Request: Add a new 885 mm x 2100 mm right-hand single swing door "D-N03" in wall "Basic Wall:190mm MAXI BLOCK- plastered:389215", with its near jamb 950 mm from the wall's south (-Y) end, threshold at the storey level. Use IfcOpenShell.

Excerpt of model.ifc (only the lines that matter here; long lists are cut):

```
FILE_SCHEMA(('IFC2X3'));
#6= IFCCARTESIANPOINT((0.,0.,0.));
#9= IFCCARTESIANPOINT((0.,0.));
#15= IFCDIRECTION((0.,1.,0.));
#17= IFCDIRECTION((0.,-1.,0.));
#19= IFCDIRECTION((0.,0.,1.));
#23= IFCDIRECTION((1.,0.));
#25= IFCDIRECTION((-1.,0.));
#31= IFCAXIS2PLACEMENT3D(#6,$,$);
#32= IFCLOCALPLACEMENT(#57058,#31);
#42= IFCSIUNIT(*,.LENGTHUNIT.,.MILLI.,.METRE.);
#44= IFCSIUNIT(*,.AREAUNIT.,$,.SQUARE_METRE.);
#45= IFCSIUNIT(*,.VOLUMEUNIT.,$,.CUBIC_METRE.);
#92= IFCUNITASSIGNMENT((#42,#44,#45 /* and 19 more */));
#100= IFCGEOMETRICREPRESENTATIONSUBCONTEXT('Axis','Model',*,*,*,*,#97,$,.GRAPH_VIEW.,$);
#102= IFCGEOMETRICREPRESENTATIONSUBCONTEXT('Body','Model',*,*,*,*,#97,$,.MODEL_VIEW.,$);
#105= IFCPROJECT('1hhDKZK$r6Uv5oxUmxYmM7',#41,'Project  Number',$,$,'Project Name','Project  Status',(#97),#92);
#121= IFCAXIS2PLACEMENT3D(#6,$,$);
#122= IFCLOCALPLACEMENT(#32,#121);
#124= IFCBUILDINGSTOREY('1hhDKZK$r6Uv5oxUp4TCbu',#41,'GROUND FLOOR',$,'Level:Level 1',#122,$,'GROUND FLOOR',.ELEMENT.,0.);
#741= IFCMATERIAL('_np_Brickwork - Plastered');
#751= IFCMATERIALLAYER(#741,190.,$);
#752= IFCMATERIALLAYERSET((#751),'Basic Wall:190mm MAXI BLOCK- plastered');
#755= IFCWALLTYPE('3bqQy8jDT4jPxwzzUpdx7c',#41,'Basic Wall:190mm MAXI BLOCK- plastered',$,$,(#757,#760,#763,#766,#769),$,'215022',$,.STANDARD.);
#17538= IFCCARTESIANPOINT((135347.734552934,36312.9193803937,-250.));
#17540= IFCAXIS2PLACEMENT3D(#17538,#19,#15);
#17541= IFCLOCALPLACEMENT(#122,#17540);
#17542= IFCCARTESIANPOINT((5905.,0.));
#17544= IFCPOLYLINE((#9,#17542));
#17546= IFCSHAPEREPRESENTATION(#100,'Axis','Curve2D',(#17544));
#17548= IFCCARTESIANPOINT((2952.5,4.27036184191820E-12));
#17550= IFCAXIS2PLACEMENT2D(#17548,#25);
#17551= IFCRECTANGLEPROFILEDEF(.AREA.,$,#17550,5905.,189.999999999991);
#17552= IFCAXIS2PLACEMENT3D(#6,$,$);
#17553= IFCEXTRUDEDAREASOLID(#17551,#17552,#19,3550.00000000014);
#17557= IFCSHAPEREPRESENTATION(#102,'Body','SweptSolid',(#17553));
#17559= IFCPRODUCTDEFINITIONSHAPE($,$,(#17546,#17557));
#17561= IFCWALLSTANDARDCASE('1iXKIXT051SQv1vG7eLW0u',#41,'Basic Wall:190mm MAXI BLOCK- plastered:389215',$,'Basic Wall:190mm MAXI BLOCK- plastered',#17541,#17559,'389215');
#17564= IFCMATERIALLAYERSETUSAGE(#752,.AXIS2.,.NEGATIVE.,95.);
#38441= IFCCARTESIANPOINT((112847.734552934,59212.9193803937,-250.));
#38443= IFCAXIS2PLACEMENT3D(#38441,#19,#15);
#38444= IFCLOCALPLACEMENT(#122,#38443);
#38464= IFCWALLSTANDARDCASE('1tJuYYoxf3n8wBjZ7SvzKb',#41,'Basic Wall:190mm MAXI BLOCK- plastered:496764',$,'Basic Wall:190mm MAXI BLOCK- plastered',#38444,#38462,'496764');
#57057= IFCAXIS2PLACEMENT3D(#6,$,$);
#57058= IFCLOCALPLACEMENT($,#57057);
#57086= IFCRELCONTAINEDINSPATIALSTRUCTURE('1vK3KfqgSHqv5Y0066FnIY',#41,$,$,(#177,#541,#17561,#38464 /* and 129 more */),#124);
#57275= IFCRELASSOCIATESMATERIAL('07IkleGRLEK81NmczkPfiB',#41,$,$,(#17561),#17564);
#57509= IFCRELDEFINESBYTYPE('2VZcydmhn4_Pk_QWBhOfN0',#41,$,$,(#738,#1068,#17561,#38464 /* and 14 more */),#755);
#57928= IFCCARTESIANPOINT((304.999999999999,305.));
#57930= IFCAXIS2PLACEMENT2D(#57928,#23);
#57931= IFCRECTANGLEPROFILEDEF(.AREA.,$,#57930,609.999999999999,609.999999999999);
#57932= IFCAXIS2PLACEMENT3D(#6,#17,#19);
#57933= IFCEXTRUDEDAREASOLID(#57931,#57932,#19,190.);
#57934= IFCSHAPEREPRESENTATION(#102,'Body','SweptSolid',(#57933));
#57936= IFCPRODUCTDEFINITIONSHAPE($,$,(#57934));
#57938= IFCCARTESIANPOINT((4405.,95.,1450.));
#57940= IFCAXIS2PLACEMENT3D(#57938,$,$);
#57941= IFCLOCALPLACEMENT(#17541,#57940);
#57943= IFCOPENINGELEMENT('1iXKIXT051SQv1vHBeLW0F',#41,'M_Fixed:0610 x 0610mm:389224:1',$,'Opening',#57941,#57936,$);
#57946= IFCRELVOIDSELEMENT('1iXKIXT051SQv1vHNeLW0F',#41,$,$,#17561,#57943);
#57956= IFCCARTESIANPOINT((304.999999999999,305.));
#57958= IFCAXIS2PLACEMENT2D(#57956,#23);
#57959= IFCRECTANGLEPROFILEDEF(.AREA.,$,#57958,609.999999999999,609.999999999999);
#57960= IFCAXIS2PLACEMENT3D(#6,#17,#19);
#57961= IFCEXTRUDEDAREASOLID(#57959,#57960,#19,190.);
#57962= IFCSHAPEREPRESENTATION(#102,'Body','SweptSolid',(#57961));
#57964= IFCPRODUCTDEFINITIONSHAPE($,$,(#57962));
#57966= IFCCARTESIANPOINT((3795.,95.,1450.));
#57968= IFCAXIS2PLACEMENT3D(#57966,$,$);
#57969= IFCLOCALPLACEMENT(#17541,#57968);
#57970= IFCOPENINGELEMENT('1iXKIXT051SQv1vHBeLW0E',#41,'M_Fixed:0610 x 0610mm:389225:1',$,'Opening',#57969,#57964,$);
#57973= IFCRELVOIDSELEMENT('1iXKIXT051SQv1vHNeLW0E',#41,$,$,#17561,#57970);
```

```python
import numpy as np
import ifcopenshell
import ifcopenshell.api.feature
import ifcopenshell.api.geometry
import ifcopenshell.api.root
import ifcopenshell.api.spatial
import ifcopenshell.api.type
import ifcopenshell.geom
import ifcopenshell.util.element
import ifcopenshell.util.placement
import ifcopenshell.util.representation
import ifcopenshell.util.shape
import ifcopenshell.util.unit

model = ifcopenshell.open("model.ifc")
unit_scale = ifcopenshell.util.unit.calculate_unit_scale(model)
settings = ifcopenshell.geom.settings()


def volume(element):
    """Net volume in cubic metres, openings subtracted."""
    shape = ifcopenshell.geom.create_shape(settings, element)
    return ifcopenshell.util.shape.get_volume(shape.geometry)


wall = model.by_id(17561)
storey = ifcopenshell.util.element.get_container(wall, ifc_class="IfcBuildingStorey")
context = ifcopenshell.util.representation.get_context(model, "Model", "Body", "MODEL_VIEW")
before = volume(wall)

width, height, from_end, sill = 0.885, 2.1, 0.95, 0.0  # metres

# The wall runs along its own X axis, and the end named is its -X end.
wall_shape = ifcopenshell.geom.create_shape(settings, wall)
x, y, z = ifcopenshell.util.shape.get_vertices(wall_shape.geometry).T
start = x.min() + from_end
face, thickness = float(y.min()), float(y.max() - y.min())
wall_matrix = ifcopenshell.util.placement.get_local_placement(wall.ObjectPlacement)
level = ifcopenshell.util.placement.get_local_placement(storey.ObjectPlacement)[2, 3]


def in_wall(x, y):
    """Placement at x, y metres in the wall's axes, at sill height."""
    matrix = wall_matrix.copy()
    matrix[:, 3] = wall_matrix @ np.array([x / unit_scale, y / unit_scale, 0.0, 1.0])
    matrix[2, 3] = level + sill / unit_scale
    return matrix


# Opening: a box that overshoots both wall faces by 50 mm.
opening = ifcopenshell.api.root.create_entity(model, ifc_class="IfcOpeningElement")
box = ifcopenshell.api.geometry.add_wall_representation(
    model, context=context, length=width, height=height, thickness=thickness + 0.1
)
ifcopenshell.api.geometry.assign_representation(model, product=opening, representation=box)
ifcopenshell.api.geometry.edit_object_placement(model, product=opening, matrix=in_wall(start, face - 0.05), is_si=False)
ifcopenshell.api.feature.add_feature(model, feature=opening, element=wall)

door = ifcopenshell.api.root.create_entity(model, ifc_class="IfcDoor", name="D-N03")
door.OverallWidth, door.OverallHeight = width / unit_scale, height / unit_scale
body = ifcopenshell.api.geometry.add_door_representation(
    model,
    context=context,
    overall_width=door.OverallWidth,
    overall_height=door.OverallHeight,
    operation_type="SINGLE_SWING_RIGHT",
    lining_properties={"LiningDepth": thickness / unit_scale, "ThresholdDepth": thickness / unit_scale},
)
ifcopenshell.api.geometry.assign_representation(model, product=door, representation=body)
ifcopenshell.api.spatial.assign_container(model, products=[door], relating_structure=storey)
fills = ifcopenshell.api.feature.add_filling(model, opening=opening, element=door)
fills.OwnerHistory = door.OwnerHistory  # required in IFC2X3

# IFC2X3 keeps the operation on the door style.
style = ifcopenshell.api.root.create_entity(model, ifc_class="IfcDoorStyle", name="D-N03")
style.OperationType, style.ConstructionType = "SINGLE_SWING_RIGHT", "NOTDEFINED"
style.ParameterTakesPrecedence = style.Sizeable = False
ifcopenshell.api.type.assign_type(model, related_objects=[door], relating_type=style)

# The lining spans the wall, so the door starts at the wall face.
ifcopenshell.api.geometry.edit_object_placement(model, product=door, matrix=in_wall(start, face), is_si=False)

after = volume(wall)

print(f"wall volume {before:.3f} -> {after:.3f} m3")

model.write("model_updated.ifc")
```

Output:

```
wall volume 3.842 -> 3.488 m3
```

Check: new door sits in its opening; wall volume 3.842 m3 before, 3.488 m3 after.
